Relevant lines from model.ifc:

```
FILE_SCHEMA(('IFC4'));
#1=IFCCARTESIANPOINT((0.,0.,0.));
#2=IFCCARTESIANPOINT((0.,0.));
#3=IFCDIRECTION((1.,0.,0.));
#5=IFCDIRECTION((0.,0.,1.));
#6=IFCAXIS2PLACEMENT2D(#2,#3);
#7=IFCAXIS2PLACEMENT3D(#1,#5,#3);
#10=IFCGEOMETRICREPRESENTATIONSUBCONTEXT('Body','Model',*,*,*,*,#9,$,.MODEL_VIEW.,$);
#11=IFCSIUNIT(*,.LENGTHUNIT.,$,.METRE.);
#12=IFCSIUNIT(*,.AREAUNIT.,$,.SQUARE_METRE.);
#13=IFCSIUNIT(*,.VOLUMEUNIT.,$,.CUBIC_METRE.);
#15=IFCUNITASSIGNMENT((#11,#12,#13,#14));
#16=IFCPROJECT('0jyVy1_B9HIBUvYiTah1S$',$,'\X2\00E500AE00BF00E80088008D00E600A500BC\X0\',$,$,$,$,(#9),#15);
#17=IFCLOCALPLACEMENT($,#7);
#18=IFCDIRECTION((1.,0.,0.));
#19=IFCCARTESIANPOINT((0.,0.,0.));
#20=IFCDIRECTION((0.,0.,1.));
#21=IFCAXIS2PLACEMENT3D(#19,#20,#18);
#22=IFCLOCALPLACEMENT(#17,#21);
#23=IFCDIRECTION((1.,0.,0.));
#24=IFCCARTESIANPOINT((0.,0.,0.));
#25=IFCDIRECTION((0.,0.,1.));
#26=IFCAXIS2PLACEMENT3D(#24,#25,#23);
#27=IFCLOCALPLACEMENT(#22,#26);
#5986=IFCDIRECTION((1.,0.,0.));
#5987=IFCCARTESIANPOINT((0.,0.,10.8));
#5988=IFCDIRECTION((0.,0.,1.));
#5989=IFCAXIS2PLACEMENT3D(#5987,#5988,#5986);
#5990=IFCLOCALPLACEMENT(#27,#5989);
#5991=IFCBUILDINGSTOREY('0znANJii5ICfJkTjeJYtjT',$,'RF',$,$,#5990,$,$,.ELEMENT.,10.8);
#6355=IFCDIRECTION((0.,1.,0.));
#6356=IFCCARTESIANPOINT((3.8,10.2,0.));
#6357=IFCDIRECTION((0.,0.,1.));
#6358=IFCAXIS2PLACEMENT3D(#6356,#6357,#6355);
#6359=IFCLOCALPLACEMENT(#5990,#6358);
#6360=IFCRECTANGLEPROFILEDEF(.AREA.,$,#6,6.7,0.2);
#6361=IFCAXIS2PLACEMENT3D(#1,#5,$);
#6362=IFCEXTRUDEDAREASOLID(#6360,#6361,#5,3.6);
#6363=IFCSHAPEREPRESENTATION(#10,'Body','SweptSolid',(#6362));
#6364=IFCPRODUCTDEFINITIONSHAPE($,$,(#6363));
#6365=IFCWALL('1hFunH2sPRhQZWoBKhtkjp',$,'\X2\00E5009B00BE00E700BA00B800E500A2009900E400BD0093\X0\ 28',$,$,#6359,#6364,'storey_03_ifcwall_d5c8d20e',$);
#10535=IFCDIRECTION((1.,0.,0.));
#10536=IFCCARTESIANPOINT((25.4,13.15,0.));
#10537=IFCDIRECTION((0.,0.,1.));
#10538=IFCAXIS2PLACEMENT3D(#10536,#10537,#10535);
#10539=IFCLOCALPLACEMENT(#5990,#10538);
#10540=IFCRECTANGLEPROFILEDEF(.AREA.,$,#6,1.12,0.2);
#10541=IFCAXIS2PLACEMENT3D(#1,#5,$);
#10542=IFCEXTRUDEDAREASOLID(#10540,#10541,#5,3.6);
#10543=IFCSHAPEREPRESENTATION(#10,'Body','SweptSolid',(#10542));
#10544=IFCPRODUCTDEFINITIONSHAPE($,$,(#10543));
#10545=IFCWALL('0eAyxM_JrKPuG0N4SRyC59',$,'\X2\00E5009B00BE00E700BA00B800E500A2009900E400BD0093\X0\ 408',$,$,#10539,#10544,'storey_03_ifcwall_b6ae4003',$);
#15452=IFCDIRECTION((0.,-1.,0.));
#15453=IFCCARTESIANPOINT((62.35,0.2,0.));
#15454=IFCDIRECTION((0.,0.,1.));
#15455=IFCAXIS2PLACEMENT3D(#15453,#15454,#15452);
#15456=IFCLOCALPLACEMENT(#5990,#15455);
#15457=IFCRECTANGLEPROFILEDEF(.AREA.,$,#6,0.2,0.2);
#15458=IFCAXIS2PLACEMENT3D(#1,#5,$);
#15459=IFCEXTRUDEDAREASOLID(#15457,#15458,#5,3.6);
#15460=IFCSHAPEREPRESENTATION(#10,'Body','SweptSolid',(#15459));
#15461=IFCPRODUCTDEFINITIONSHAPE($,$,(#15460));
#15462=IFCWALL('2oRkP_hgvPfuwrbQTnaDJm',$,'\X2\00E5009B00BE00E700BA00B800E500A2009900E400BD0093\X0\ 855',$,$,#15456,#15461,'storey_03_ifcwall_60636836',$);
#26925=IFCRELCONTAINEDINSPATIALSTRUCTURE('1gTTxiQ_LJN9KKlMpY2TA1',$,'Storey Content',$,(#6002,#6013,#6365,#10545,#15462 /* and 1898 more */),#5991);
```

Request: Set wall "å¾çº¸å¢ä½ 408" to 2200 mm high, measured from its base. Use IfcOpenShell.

```python
import ifcopenshell
import ifcopenshell.geom
import ifcopenshell.util.representation
import ifcopenshell.util.shape
import ifcopenshell.util.unit

model = ifcopenshell.open("model.ifc")
unit_scale = ifcopenshell.util.unit.calculate_unit_scale(model)
settings = ifcopenshell.geom.settings()


def volume(element):
    """Net volume in cubic metres, openings subtracted."""
    shape = ifcopenshell.geom.create_shape(settings, element)
    return ifcopenshell.util.shape.get_volume(shape.geometry)


wall = model.by_guid("0eAyxM_JrKPuG0N4SRyC59")
before = volume(wall)

body = ifcopenshell.util.representation.get_representation(wall, "Model", "Body")
solid = body.Items[0]
old_height = solid.Depth
solid.Depth = 2.2 / unit_scale
after = volume(wall)

print(f"height {old_height:g} -> {solid.Depth:g}, volume {before:.3f} -> {after:.3f} m3")

model.write("model_rev.ifc")
```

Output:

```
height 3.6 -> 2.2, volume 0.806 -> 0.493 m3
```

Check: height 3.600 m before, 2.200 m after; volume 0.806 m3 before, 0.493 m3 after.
